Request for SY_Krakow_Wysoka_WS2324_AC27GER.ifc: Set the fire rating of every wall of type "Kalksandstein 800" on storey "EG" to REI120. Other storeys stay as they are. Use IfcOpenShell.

First a look at what the model holds.

```python
import ifcopenshell
import ifcopenshell.util.element

model = ifcopenshell.open("SY_Krakow_Wysoka_WS2324_AC27GER.ifc")
print(model.schema)
storey = next(s for s in model.by_type("IfcBuildingStorey") if s.Name == "EG")
walls = [e for e in ifcopenshell.util.element.get_decomposition(storey) if e.is_a("IfcWall")]
seen = {}
for e in walls:
    element_type = ifcopenshell.util.element.get_type(e)
    key = (element_type.Name if element_type != e and element_type else None, ifcopenshell.util.element.get_pset(e, "Pset_WallCommon", "FireRating"))
    seen[key] = seen.get(key, 0) + 1
for (name, value), count in sorted(seen.items(), key=str):
    print(count, "x", name, "|", value)
```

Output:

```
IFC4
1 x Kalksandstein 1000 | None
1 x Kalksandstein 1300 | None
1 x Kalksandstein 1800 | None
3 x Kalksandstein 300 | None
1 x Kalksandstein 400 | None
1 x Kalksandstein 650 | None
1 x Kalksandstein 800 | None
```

```python
import ifcopenshell
import ifcopenshell.api.pset
import ifcopenshell.util.element

model = ifcopenshell.open("SY_Krakow_Wysoka_WS2324_AC27GER.ifc")

storey = next(s for s in model.by_type("IfcBuildingStorey") if s.Name == "EG")
walls = [e for e in ifcopenshell.util.element.get_decomposition(storey) if e.is_a("IfcWall")]

count = 0
for e in walls:
    element_type = ifcopenshell.util.element.get_type(e)
    if element_type in (None, e) or element_type.Name != "Kalksandstein 800":
        continue
    # add_pset returns the element's existing set when there is one.
    pset = ifcopenshell.api.pset.add_pset(model, product=e, name="Pset_WallCommon")
    ifcopenshell.api.pset.edit_pset(model, pset=pset, properties={"FireRating": "REI120"})
    count += 1

print(count, "walls updated")

model.write("SY_Krakow_Wysoka_WS2324_AC27GER_v2.ifc")
```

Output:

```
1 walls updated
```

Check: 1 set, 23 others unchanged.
